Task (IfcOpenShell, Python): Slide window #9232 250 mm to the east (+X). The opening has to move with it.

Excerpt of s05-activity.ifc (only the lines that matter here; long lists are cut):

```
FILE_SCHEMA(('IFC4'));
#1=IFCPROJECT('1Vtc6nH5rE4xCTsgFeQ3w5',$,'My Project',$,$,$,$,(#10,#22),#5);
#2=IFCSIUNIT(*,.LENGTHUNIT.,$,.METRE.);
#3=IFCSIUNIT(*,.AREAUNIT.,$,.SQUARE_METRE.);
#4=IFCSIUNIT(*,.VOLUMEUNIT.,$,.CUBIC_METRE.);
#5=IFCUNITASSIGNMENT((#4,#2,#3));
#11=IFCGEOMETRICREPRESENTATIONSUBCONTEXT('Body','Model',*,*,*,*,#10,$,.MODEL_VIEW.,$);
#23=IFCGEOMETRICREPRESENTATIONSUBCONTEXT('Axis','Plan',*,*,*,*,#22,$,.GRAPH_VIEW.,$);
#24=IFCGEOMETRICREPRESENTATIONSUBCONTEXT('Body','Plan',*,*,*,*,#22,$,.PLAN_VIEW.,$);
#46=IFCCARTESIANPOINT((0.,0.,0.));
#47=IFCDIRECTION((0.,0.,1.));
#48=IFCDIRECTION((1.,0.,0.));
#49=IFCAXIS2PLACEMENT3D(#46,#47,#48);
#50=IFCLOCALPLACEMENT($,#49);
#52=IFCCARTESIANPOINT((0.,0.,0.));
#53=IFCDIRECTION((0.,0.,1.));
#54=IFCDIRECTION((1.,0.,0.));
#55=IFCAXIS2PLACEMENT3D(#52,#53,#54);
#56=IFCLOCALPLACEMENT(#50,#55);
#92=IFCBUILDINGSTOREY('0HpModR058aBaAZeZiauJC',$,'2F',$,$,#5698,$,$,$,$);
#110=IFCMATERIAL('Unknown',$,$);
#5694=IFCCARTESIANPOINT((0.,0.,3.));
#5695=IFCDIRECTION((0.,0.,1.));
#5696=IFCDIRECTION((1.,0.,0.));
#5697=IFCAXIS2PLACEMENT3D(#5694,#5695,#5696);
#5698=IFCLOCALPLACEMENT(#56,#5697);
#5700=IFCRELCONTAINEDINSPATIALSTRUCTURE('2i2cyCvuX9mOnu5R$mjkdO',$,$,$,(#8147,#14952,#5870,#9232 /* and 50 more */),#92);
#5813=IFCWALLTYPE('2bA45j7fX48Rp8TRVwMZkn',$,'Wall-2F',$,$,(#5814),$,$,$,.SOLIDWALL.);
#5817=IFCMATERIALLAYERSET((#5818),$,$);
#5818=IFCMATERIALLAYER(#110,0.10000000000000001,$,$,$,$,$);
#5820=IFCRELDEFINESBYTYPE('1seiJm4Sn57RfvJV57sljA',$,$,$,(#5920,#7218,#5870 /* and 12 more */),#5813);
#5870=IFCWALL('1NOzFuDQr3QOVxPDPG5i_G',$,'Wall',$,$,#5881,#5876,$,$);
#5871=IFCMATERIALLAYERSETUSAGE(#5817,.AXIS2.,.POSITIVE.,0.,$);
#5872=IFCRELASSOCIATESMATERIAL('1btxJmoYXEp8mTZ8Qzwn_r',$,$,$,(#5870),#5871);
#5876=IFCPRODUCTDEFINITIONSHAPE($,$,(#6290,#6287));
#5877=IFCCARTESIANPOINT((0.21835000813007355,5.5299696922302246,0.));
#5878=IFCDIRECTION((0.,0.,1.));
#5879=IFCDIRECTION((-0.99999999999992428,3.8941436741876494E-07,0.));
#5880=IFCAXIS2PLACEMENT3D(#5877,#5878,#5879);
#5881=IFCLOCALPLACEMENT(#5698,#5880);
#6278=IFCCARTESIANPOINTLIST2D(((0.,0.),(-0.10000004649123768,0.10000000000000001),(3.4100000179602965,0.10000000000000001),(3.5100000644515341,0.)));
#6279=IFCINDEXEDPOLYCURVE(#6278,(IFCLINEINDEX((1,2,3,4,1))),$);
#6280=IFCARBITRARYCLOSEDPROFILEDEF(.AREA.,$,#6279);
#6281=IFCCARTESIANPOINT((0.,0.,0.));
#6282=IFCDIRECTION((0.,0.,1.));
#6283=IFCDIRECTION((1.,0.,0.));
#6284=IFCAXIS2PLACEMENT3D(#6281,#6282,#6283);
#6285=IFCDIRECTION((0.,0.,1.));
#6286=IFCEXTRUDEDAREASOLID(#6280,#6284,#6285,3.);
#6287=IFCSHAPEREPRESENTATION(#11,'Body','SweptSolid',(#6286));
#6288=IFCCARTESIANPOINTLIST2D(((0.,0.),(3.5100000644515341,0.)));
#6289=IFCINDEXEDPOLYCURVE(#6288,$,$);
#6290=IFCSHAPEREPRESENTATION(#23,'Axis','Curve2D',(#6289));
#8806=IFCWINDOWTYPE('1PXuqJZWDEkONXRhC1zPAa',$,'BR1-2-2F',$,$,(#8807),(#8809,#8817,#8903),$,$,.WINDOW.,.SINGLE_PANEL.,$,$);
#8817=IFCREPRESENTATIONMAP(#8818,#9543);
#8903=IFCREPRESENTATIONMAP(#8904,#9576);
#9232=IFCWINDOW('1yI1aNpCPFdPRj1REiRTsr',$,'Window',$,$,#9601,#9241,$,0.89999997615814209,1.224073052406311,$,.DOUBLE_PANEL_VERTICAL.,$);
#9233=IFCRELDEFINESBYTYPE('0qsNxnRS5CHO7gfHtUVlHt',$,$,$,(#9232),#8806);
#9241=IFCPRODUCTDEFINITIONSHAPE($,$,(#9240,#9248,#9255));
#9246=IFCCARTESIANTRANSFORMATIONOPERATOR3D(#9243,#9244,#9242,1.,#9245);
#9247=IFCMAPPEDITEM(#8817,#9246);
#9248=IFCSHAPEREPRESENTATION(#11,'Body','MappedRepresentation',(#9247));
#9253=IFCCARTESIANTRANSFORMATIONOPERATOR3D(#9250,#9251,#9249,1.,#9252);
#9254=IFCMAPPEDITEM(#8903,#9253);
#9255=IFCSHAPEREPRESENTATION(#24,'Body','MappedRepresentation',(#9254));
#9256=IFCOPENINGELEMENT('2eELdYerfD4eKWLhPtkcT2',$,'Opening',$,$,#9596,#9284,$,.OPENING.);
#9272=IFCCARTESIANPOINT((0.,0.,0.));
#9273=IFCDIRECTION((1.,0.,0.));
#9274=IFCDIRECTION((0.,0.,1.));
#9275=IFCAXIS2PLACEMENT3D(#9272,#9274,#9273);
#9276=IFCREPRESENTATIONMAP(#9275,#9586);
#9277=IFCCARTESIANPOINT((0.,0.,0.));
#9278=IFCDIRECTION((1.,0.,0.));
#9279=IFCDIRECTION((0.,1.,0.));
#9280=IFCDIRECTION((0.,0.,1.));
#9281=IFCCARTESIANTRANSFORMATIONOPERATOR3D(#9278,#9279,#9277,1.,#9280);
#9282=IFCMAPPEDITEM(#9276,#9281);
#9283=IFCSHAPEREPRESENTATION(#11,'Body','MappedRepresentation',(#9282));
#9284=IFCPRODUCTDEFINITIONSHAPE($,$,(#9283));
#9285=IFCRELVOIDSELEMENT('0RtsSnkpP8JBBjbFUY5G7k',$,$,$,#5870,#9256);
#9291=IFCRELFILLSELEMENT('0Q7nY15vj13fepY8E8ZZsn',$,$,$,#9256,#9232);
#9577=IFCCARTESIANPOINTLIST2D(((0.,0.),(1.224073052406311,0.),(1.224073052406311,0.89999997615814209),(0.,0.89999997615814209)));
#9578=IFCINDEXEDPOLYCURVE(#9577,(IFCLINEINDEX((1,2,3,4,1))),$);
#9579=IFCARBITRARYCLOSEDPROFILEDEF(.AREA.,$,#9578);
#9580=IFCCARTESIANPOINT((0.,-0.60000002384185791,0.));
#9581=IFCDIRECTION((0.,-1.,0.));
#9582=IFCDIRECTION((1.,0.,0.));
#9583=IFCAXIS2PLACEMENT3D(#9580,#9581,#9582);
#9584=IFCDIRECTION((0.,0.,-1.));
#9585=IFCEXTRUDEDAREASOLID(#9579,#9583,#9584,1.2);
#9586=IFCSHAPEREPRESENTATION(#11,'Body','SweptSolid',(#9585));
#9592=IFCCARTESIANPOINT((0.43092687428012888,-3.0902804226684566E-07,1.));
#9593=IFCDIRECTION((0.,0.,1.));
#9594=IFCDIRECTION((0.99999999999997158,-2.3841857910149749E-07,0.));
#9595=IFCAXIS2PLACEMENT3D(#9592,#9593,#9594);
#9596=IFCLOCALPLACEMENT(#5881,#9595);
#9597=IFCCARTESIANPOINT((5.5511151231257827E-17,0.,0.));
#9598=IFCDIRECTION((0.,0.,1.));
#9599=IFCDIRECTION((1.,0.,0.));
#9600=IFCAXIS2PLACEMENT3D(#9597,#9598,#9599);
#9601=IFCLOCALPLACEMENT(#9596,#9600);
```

```python
import ifcopenshell
import ifcopenshell.api.geometry
import ifcopenshell.util.placement
import ifcopenshell.util.unit

model = ifcopenshell.open("s05-activity.ifc")
unit_scale = ifcopenshell.util.unit.calculate_unit_scale(model)

window = model.by_id(9232)
opening = window.FillsVoids[0].RelatingOpeningElement
wall = opening.VoidsElements[0].RelatingBuildingElement

wall_matrix = ifcopenshell.util.placement.get_local_placement(wall.ObjectPlacement)
shift = wall_matrix[:3, 0] * -0.25 / unit_scale
before = ifcopenshell.util.placement.get_local_placement(window.ObjectPlacement)[:3, 3].copy()

# The window is placed relative to its opening, so it follows when the opening moves.
matrix = ifcopenshell.util.placement.get_local_placement(opening.ObjectPlacement)
matrix[:3, 3] += shift
ifcopenshell.api.geometry.edit_object_placement(
    model, product=opening, matrix=matrix, is_si=False, should_transform_children=True
)

after = ifcopenshell.util.placement.get_local_placement(window.ObjectPlacement)[:3, 3]
print("window moved by", (after - before).round(3) + 0.0)

model.write("s05-activity_rev.ifc")
```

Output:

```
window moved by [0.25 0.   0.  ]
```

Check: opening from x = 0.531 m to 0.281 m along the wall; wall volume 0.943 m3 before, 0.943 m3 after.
